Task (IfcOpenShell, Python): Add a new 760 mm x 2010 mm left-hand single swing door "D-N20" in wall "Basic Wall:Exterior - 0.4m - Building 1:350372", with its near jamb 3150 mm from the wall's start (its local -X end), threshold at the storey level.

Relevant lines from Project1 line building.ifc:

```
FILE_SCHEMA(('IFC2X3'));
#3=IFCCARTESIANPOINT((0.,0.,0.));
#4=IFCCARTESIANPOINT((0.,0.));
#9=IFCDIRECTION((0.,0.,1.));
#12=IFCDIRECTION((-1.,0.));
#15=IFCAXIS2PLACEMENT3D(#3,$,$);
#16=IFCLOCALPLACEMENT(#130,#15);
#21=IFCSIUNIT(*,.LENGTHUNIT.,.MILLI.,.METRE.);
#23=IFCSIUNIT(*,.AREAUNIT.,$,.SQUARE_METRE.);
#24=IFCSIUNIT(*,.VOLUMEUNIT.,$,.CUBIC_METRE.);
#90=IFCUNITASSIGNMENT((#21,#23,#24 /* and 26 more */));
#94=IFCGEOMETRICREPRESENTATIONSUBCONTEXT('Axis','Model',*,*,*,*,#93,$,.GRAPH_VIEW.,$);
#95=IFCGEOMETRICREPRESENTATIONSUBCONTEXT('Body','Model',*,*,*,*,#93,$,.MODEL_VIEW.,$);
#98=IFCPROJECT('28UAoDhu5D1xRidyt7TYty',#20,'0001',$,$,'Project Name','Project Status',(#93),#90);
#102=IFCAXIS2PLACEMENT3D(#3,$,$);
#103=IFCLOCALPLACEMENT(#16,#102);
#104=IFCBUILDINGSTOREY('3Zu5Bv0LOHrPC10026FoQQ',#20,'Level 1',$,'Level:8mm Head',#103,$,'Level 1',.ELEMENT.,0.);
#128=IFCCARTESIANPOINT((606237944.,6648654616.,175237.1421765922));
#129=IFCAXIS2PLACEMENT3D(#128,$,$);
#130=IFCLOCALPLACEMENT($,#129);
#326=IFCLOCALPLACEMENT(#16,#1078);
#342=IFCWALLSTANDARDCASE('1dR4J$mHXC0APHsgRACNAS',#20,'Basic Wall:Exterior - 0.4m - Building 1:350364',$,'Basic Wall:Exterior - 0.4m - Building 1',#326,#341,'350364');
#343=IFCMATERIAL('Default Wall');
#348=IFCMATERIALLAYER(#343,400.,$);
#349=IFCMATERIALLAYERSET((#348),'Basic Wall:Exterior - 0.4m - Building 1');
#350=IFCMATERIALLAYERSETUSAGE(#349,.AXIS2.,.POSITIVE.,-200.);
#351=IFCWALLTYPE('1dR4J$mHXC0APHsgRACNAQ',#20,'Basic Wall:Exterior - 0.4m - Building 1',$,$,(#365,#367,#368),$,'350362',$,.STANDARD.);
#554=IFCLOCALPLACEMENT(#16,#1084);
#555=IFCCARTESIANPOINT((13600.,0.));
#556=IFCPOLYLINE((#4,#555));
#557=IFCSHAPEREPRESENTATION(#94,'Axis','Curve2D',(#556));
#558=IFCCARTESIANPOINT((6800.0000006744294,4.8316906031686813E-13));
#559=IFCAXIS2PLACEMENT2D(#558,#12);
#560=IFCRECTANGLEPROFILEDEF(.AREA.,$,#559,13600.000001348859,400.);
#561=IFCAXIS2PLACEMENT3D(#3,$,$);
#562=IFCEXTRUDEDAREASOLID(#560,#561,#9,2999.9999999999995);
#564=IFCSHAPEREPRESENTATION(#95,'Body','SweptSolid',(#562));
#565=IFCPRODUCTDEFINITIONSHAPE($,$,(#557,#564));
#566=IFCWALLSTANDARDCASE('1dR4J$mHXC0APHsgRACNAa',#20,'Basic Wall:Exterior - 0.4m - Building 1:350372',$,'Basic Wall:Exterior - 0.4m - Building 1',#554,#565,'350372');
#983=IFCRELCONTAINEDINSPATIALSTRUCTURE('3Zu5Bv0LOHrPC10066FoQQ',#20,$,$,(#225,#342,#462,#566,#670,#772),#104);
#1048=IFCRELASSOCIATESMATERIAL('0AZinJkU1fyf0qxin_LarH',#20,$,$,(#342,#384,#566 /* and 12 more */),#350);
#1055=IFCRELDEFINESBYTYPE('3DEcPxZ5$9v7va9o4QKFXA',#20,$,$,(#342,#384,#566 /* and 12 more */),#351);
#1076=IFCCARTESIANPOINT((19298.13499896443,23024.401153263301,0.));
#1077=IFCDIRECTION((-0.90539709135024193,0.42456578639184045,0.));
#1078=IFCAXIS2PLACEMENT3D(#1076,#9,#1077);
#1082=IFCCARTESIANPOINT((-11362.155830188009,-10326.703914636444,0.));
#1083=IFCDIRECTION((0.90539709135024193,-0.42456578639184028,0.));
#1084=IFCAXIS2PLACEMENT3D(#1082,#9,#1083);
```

```python
import numpy as np
import ifcopenshell
import ifcopenshell.api.feature
import ifcopenshell.api.geometry
import ifcopenshell.api.root
import ifcopenshell.api.spatial
import ifcopenshell.api.type
import ifcopenshell.geom
import ifcopenshell.util.element
import ifcopenshell.util.placement
import ifcopenshell.util.representation
import ifcopenshell.util.shape
import ifcopenshell.util.unit

model = ifcopenshell.open("Project1 line building.ifc")
unit_scale = ifcopenshell.util.unit.calculate_unit_scale(model)
settings = ifcopenshell.geom.settings()


def volume(element):
    """Net volume in cubic metres, openings subtracted."""
    shape = ifcopenshell.geom.create_shape(settings, element)
    return ifcopenshell.util.shape.get_volume(shape.geometry)


wall = model.by_guid("1dR4J$mHXC0APHsgRACNAa")
storey = ifcopenshell.util.element.get_container(wall, ifc_class="IfcBuildingStorey")
context = ifcopenshell.util.representation.get_context(model, "Model", "Body", "MODEL_VIEW")
before = volume(wall)

width, height, from_end, sill = 0.76, 2.01, 3.15, 0.0  # metres

# The wall runs along its own X axis, and the end named is its -X end.
wall_shape = ifcopenshell.geom.create_shape(settings, wall)
x, y, z = ifcopenshell.util.shape.get_vertices(wall_shape.geometry).T
start = x.min() + from_end
face, thickness = float(y.min()), float(y.max() - y.min())
wall_matrix = ifcopenshell.util.placement.get_local_placement(wall.ObjectPlacement)
level = ifcopenshell.util.placement.get_local_placement(storey.ObjectPlacement)[2, 3]


def in_wall(x, y):
    """Placement at x, y metres in the wall's axes, at sill height."""
    matrix = wall_matrix.copy()
    matrix[:, 3] = wall_matrix @ np.array([x / unit_scale, y / unit_scale, 0.0, 1.0])
    matrix[2, 3] = level + sill / unit_scale
    return matrix


# Opening: a box that overshoots both wall faces by 50 mm.
opening = ifcopenshell.api.root.create_entity(model, ifc_class="IfcOpeningElement")
box = ifcopenshell.api.geometry.add_wall_representation(
    model, context=context, length=width, height=height, thickness=thickness + 0.1
)
ifcopenshell.api.geometry.assign_representation(model, product=opening, representation=box)
ifcopenshell.api.geometry.edit_object_placement(model, product=opening, matrix=in_wall(start, face - 0.05), is_si=False)
ifcopenshell.api.feature.add_feature(model, feature=opening, element=wall)

door = ifcopenshell.api.root.create_entity(model, ifc_class="IfcDoor", name="D-N20")
door.OverallWidth, door.OverallHeight = width / unit_scale, height / unit_scale
body = ifcopenshell.api.geometry.add_door_representation(
    model,
    context=context,
    overall_width=door.OverallWidth,
    overall_height=door.OverallHeight,
    operation_type="SINGLE_SWING_LEFT",
    lining_properties={"LiningDepth": thickness / unit_scale, "ThresholdDepth": thickness / unit_scale},
)
ifcopenshell.api.geometry.assign_representation(model, product=door, representation=body)
ifcopenshell.api.spatial.assign_container(model, products=[door], relating_structure=storey)
fills = ifcopenshell.api.feature.add_filling(model, opening=opening, element=door)
fills.OwnerHistory = door.OwnerHistory  # required in IFC2X3

# IFC2X3 keeps the operation on the door style.
style = ifcopenshell.api.root.create_entity(model, ifc_class="IfcDoorStyle", name="D-N20")
style.OperationType, style.ConstructionType = "SINGLE_SWING_LEFT", "NOTDEFINED"
style.ParameterTakesPrecedence = style.Sizeable = False
ifcopenshell.api.type.assign_type(model, related_objects=[door], relating_type=style)

# The lining spans the wall, so the door starts at the wall face.
ifcopenshell.api.geometry.edit_object_placement(model, product=door, matrix=in_wall(start, face), is_si=False)

after = volume(wall)

print(f"wall volume {before:.3f} -> {after:.3f} m3")

model.write("Project1 line building_edited.ifc")
```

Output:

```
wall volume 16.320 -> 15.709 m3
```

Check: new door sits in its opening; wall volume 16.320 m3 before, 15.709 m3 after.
